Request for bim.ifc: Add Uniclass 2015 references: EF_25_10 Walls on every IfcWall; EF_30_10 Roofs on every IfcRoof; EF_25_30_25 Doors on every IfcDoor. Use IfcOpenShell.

First a look at what the model holds.

```python
import ifcopenshell

model = ifcopenshell.open("bim.ifc")
print(model.schema)
print("classifications:", [c.Name for c in model.by_type("IfcClassification")])
for ifc_class in ("IfcDoor", "IfcRoof", "IfcStair", "IfcWall", "IfcWindow"):
    print(ifc_class, len(model.by_type(ifc_class)))
```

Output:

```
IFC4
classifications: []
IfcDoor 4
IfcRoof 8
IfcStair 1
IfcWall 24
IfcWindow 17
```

```python
import ifcopenshell
import ifcopenshell.api.classification

model = ifcopenshell.open("bim.ifc")

system = ifcopenshell.api.classification.add_classification(model, classification="Uniclass 2015")

codes = {
    "IfcWall": ("EF_25_10", "Walls"),
    "IfcRoof": ("EF_30_10", "Roofs"),
    "IfcDoor": ("EF_25_30_25", "Doors"),
}
for ifc_class, (code, name) in codes.items():
    products = model.by_type(ifc_class)
    ifcopenshell.api.classification.add_reference(
        model, products=products, classification=system, identification=code, name=name
    )
    print(code, len(products))

model.write("bim_edited.ifc")
```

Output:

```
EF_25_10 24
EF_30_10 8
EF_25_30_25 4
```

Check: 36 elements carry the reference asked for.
